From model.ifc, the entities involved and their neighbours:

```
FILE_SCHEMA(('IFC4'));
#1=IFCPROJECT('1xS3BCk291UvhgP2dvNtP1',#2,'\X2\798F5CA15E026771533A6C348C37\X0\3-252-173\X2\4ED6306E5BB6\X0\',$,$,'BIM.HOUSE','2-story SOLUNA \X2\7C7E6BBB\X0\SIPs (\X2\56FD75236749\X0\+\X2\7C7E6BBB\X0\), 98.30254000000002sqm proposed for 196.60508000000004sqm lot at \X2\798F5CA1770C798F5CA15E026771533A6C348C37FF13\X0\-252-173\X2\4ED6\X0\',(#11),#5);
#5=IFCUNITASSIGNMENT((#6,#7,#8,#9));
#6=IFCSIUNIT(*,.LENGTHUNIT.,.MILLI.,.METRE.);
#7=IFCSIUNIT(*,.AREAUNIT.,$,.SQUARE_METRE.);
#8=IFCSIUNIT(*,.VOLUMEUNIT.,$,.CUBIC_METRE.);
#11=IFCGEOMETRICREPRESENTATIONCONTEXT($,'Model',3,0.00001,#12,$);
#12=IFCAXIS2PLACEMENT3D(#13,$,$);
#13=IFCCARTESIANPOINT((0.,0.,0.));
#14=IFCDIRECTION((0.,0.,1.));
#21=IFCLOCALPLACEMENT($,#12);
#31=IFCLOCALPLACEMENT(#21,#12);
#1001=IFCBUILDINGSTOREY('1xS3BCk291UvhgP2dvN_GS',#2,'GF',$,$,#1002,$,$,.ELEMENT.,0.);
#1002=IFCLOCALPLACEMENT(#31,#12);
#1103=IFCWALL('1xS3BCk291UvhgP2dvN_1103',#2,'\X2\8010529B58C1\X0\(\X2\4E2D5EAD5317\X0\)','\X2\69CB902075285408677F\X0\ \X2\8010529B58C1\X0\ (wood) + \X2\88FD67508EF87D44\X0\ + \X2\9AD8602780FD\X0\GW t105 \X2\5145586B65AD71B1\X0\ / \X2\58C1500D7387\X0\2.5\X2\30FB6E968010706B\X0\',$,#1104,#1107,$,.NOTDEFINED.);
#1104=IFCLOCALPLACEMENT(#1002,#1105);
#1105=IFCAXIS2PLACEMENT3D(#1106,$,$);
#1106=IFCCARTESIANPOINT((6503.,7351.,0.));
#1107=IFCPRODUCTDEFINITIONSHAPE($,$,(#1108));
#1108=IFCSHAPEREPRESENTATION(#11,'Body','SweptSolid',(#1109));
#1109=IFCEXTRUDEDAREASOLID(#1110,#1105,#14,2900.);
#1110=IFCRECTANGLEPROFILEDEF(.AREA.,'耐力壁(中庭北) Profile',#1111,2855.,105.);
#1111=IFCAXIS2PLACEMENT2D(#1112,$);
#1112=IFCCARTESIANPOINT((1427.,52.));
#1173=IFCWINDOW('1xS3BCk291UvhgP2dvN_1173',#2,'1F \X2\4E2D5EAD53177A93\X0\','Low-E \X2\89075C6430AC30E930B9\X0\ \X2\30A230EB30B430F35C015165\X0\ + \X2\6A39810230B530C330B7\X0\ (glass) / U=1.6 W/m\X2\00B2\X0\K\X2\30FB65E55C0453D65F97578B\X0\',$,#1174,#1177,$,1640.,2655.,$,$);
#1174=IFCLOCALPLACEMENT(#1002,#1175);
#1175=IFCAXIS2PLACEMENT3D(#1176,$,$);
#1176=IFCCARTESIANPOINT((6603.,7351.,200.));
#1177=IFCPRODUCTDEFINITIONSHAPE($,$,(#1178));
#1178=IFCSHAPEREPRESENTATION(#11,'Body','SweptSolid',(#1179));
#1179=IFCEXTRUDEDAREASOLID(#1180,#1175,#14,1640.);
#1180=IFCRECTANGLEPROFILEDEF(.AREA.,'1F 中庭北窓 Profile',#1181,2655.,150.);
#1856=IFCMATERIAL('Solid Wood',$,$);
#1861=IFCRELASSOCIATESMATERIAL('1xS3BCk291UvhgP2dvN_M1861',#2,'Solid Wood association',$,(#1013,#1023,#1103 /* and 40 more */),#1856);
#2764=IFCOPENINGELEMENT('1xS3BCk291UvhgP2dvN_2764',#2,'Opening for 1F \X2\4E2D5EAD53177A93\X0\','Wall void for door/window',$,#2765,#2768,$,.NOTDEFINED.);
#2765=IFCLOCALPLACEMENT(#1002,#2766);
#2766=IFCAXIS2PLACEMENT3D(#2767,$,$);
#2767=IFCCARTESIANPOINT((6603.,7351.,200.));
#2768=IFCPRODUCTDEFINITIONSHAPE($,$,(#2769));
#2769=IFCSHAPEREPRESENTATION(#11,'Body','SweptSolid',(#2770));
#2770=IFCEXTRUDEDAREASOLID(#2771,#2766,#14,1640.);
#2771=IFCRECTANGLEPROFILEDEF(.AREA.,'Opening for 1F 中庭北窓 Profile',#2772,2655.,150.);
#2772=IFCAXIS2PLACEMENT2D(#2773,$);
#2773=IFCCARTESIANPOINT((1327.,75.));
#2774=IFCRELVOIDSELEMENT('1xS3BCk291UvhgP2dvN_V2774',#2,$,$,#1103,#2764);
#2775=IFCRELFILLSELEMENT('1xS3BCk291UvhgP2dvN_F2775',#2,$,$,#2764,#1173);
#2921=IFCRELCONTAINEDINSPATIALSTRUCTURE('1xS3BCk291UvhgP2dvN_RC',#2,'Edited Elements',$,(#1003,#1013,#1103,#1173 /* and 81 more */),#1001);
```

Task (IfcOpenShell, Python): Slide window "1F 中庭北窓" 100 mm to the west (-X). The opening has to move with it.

```python
import ifcopenshell
import ifcopenshell.api.geometry
import ifcopenshell.util.placement
import ifcopenshell.util.unit

model = ifcopenshell.open("model.ifc")
unit_scale = ifcopenshell.util.unit.calculate_unit_scale(model)

window = model.by_id(1173)
opening = window.FillsVoids[0].RelatingOpeningElement
wall = opening.VoidsElements[0].RelatingBuildingElement

wall_matrix = ifcopenshell.util.placement.get_local_placement(wall.ObjectPlacement)
shift = wall_matrix[:3, 0] * -0.1 / unit_scale
before = ifcopenshell.util.placement.get_local_placement(window.ObjectPlacement)[:3, 3].copy()

# The window is not placed relative to its opening, so move both.
for product in (opening, window):
    matrix = ifcopenshell.util.placement.get_local_placement(product.ObjectPlacement)
    matrix[:3, 3] += shift
    ifcopenshell.api.geometry.edit_object_placement(model, product=product, matrix=matrix, is_si=False)

after = ifcopenshell.util.placement.get_local_placement(window.ObjectPlacement)[:3, 3]
print("window moved by", (after - before).round(3) + 0.0)

model.write("model_v2.ifc")
```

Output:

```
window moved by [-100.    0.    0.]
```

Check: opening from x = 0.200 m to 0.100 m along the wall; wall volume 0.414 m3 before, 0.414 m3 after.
